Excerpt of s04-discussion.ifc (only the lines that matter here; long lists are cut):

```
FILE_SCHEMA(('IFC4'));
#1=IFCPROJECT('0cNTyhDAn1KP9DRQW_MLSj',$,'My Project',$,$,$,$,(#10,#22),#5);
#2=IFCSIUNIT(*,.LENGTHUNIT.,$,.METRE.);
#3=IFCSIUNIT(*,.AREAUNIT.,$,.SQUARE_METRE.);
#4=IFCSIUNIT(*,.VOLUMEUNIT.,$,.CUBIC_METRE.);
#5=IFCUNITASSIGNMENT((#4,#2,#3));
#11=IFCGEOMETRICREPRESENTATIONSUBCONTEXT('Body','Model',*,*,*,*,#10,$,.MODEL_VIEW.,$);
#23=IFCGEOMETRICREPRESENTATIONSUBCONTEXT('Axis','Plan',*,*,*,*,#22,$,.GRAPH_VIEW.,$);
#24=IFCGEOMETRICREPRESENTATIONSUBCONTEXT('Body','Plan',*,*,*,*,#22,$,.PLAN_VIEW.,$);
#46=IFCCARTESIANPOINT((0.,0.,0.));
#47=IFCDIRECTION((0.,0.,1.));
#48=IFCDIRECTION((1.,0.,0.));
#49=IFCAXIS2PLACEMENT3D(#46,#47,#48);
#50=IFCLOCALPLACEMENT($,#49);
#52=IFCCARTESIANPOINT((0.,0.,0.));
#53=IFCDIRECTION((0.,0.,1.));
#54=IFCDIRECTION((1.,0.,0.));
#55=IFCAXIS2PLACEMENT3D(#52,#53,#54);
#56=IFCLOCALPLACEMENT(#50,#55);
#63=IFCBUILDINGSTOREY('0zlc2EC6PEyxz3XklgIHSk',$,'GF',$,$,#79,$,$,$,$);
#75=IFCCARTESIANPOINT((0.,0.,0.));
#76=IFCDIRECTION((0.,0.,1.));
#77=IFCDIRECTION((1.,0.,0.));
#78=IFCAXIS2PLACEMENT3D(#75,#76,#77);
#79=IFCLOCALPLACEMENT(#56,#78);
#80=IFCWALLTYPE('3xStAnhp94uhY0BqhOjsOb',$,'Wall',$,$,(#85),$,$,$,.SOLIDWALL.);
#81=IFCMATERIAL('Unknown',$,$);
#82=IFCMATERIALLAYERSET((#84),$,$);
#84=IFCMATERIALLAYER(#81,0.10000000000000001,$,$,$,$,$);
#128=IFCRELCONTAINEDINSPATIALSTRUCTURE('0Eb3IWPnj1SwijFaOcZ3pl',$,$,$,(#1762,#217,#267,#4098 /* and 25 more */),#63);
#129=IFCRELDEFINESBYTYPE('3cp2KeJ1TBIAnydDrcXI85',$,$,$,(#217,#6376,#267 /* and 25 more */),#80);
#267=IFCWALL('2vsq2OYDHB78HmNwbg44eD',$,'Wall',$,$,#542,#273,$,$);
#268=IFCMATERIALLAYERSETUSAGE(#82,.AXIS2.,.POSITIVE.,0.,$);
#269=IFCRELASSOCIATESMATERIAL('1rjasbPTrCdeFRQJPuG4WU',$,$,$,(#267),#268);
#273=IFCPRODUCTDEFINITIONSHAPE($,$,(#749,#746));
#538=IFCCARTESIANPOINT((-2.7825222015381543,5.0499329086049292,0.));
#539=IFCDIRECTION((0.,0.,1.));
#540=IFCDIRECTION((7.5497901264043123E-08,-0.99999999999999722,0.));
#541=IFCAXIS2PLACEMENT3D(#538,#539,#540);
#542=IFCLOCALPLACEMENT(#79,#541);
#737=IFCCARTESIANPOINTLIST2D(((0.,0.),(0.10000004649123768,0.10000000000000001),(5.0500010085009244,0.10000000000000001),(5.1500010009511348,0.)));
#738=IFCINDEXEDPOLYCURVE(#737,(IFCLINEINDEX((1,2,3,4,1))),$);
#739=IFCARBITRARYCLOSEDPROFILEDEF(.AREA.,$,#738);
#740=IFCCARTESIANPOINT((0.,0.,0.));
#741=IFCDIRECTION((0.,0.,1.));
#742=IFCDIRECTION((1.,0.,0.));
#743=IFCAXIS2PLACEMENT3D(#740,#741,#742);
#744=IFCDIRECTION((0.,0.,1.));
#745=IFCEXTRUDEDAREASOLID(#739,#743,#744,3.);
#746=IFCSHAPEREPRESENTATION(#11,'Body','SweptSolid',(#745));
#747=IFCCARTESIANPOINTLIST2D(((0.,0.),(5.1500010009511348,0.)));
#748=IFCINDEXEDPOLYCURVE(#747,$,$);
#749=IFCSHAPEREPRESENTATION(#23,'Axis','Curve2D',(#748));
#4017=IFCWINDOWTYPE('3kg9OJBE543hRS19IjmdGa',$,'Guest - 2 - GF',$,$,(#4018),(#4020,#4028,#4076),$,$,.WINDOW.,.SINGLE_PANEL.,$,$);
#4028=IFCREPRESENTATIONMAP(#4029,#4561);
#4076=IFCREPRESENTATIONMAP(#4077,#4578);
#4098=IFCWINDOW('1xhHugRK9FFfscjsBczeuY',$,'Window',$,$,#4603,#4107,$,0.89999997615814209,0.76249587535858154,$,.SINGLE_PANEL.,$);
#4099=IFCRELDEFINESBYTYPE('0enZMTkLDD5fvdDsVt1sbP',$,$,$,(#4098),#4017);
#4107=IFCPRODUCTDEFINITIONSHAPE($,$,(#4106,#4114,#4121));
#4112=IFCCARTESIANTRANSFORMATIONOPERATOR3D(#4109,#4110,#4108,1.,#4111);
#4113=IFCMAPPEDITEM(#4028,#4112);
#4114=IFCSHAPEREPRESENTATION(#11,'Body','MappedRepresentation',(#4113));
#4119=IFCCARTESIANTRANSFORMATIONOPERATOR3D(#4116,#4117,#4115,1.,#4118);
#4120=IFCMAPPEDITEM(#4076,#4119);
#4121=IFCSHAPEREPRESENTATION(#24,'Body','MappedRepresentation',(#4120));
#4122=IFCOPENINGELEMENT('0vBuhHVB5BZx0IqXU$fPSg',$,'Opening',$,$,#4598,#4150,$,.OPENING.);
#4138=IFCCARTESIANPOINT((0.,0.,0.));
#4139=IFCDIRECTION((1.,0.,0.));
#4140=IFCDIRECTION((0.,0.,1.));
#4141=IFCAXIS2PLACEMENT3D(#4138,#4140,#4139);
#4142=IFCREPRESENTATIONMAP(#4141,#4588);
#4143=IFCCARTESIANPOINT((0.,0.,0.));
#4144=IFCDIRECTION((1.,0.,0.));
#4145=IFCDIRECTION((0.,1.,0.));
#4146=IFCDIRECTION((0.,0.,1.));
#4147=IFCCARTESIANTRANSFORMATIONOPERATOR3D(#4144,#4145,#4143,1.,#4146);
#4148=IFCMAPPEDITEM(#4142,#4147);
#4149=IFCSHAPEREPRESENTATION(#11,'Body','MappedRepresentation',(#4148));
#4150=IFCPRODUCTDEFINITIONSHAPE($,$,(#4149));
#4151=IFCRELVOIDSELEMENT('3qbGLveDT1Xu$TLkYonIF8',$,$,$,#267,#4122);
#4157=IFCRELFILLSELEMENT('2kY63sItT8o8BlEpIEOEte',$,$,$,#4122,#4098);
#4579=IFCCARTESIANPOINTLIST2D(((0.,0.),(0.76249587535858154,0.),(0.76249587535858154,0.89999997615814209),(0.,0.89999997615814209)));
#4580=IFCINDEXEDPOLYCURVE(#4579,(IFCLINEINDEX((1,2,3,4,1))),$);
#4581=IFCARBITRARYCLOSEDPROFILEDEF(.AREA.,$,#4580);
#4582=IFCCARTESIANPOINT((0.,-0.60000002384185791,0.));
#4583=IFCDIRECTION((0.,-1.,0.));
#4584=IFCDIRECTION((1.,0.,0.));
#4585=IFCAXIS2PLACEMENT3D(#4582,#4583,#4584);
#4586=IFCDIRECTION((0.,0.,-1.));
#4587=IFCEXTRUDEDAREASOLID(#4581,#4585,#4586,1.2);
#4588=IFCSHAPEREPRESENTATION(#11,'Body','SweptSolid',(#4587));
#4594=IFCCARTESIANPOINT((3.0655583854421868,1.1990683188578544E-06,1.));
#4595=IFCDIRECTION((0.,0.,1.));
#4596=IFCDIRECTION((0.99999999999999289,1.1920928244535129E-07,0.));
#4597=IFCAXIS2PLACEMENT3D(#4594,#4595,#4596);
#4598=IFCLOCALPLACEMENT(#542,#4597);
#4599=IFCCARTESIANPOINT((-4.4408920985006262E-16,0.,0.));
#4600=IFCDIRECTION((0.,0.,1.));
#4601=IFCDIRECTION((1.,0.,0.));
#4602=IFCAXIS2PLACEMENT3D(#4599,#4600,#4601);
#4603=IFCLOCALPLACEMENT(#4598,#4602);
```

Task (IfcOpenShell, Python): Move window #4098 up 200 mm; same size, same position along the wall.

```python
import numpy as np
import ifcopenshell
import ifcopenshell.api.geometry
import ifcopenshell.util.placement
import ifcopenshell.util.unit

model = ifcopenshell.open("s04-discussion.ifc")
unit_scale = ifcopenshell.util.unit.calculate_unit_scale(model)

window = model.by_guid("1xhHugRK9FFfscjsBczeuY")
opening = window.FillsVoids[0].RelatingOpeningElement
dz = 0.2 / unit_scale

shift = np.array([0.0, 0.0, dz])
# The window is placed relative to its opening, so it follows when the opening moves.
matrix = ifcopenshell.util.placement.get_local_placement(opening.ObjectPlacement)
matrix[:3, 3] += shift
ifcopenshell.api.geometry.edit_object_placement(
    model, product=opening, matrix=matrix, is_si=False, should_transform_children=True
)

print(f"moved by {dz * unit_scale:+.3f} m")

model.write("s04-discussion_v2.ifc")
```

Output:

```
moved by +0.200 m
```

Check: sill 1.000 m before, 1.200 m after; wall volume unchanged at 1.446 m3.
